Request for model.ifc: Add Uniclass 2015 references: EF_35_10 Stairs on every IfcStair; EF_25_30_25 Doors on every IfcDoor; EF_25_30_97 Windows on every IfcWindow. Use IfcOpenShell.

First a look at what the model holds.

```python
import ifcopenshell

model = ifcopenshell.open("model.ifc")
print(model.schema)
print("classifications:", [c.Name for c in model.by_type("IfcClassification")])
for ifc_class in ("IfcDoor", "IfcRoof", "IfcStair", "IfcWall", "IfcWindow"):
    print(ifc_class, len(model.by_type(ifc_class)))
```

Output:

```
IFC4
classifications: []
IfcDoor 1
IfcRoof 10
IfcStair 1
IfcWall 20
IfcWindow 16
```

```python
import ifcopenshell
import ifcopenshell.api.classification

model = ifcopenshell.open("model.ifc")

system = ifcopenshell.api.classification.add_classification(model, classification="Uniclass 2015")

codes = {
    "IfcStair": ("EF_35_10", "Stairs"),
    "IfcDoor": ("EF_25_30_25", "Doors"),
    "IfcWindow": ("EF_25_30_97", "Windows"),
}
for ifc_class, (code, name) in codes.items():
    products = model.by_type(ifc_class)
    ifcopenshell.api.classification.add_reference(
        model, products=products, classification=system, identification=code, name=name
    )
    print(code, len(products))

model.write("model_rev.ifc")
```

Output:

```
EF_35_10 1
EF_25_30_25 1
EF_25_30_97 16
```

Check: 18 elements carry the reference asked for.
